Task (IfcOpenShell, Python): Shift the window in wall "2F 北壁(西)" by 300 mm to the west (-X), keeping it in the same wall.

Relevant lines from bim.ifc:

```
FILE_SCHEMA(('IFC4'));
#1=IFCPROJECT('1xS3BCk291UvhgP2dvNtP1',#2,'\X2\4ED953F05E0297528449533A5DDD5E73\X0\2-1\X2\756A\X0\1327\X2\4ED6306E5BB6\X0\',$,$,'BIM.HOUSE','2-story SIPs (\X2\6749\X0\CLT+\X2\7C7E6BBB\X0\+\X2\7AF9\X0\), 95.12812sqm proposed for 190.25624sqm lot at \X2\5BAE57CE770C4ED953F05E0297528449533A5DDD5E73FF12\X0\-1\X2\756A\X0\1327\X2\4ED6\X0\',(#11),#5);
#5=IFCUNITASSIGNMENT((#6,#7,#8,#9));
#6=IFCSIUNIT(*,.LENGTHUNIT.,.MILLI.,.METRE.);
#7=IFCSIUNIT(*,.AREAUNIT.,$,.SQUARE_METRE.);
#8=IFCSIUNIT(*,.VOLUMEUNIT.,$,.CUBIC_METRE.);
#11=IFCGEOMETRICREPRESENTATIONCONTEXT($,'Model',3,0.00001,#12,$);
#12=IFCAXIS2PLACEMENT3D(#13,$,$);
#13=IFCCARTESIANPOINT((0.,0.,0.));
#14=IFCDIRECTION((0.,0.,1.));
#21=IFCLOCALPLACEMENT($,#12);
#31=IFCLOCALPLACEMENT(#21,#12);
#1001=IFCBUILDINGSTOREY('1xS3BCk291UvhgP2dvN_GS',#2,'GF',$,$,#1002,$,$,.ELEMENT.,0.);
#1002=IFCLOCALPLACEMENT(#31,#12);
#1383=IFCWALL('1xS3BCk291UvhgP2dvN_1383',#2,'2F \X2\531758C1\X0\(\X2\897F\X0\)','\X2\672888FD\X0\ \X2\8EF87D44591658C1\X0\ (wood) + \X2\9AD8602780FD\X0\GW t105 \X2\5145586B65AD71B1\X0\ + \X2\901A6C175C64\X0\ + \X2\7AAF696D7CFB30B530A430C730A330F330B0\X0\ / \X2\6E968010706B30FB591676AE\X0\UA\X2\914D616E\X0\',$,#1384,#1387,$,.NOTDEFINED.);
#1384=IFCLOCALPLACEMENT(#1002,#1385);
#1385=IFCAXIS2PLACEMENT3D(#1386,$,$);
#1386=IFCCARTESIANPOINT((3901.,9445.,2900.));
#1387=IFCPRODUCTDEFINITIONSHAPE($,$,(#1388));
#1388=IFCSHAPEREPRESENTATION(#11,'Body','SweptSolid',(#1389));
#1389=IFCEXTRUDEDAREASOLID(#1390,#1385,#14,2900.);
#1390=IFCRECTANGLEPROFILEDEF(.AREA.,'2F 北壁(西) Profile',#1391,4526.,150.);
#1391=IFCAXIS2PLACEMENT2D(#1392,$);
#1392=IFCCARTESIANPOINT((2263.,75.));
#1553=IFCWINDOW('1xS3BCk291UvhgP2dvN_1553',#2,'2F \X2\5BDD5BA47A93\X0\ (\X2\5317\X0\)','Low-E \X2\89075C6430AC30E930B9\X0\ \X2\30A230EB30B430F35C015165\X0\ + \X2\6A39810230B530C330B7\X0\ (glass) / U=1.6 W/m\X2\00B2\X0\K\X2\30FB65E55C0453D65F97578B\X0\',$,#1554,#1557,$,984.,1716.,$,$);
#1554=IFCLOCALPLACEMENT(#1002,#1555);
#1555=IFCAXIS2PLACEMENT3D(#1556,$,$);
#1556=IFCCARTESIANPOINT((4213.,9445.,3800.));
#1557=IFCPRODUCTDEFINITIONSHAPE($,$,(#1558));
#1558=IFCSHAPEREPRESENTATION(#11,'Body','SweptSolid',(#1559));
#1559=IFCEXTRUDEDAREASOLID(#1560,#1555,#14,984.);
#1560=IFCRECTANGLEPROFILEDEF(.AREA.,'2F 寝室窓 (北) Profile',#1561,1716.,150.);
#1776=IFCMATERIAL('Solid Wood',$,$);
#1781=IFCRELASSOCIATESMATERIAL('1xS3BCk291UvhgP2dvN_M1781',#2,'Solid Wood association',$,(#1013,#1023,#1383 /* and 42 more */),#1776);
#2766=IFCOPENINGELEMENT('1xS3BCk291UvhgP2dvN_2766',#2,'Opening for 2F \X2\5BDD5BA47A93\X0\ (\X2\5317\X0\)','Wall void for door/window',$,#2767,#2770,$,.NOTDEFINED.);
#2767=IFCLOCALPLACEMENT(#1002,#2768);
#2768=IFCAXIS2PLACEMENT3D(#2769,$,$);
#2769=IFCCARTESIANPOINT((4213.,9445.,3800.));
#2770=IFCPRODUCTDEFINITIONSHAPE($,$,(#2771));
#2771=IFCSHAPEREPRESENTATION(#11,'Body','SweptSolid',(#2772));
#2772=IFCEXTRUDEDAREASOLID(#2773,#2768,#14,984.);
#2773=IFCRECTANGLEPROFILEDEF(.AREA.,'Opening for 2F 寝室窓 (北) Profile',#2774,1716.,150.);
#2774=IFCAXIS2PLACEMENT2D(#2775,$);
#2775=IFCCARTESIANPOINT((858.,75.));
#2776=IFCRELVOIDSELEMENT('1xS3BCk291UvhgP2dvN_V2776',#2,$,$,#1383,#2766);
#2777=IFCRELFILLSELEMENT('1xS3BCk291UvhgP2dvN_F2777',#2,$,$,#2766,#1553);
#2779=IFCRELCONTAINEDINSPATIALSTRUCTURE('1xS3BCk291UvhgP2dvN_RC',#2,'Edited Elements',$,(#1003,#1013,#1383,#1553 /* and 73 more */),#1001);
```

```python
import ifcopenshell
import ifcopenshell.api.geometry
import ifcopenshell.util.placement
import ifcopenshell.util.unit

model = ifcopenshell.open("bim.ifc")
unit_scale = ifcopenshell.util.unit.calculate_unit_scale(model)

window = model.by_id(1553)
opening = window.FillsVoids[0].RelatingOpeningElement
wall = opening.VoidsElements[0].RelatingBuildingElement

wall_matrix = ifcopenshell.util.placement.get_local_placement(wall.ObjectPlacement)
shift = wall_matrix[:3, 0] * -0.3 / unit_scale
before = ifcopenshell.util.placement.get_local_placement(window.ObjectPlacement)[:3, 3].copy()

# The window is not placed relative to its opening, so move both.
for product in (opening, window):
    matrix = ifcopenshell.util.placement.get_local_placement(product.ObjectPlacement)
    matrix[:3, 3] += shift
    ifcopenshell.api.geometry.edit_object_placement(model, product=product, matrix=matrix, is_si=False)

after = ifcopenshell.util.placement.get_local_placement(window.ObjectPlacement)[:3, 3]
print("window moved by", (after - before).round(3) + 0.0)

model.write("bim-out.ifc")
```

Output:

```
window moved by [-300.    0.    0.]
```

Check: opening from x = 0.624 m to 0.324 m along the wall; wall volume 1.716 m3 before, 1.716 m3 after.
